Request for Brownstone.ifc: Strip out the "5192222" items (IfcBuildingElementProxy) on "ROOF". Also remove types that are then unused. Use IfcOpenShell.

First a look at what the model holds.

```python
import ifcopenshell
import ifcopenshell.util.element

model = ifcopenshell.open("Brownstone.ifc")
print(model.schema)
storey = next(s for s in model.by_type("IfcBuildingStorey") if s.Name == "ROOF")
proxies = [e for e in ifcopenshell.util.element.get_decomposition(storey) if e.is_a("IfcBuildingElementProxy")]
seen = {}
for e in proxies:
    element_type = ifcopenshell.util.element.get_type(e)
    name = element_type.Name if element_type not in (None, e) else None
    seen[name] = seen.get(name, 0) + 1
for name, count in sorted(seen.items(), key=str):
    print(count, "x", name)
```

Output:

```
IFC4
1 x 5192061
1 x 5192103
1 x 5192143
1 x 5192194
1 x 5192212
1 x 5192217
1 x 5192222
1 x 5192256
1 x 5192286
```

```python
import ifcopenshell
import ifcopenshell.api.root
import ifcopenshell.util.element

model = ifcopenshell.open("Brownstone.ifc")

storey = next(s for s in model.by_type("IfcBuildingStorey") if s.Name == "ROOF")
proxies = [e for e in ifcopenshell.util.element.get_decomposition(storey) if e.is_a("IfcBuildingElementProxy")]
targets = [e for e in proxies if (t := ifcopenshell.util.element.get_type(e)) not in (None, e) and t.Name == "5192222"]
types = {ifcopenshell.util.element.get_type(e) for e in targets} - {None, *targets}

for e in targets:
    ifcopenshell.api.root.remove_product(model, product=e)
print(len(targets), "removed")

unused = [t for t in types if not ifcopenshell.util.element.get_types(t)]
for t in unused:
    ifcopenshell.api.root.remove_product(model, product=t)
print(len(unused), "unused types removed")

model.write("Brownstone_v2.ifc")
```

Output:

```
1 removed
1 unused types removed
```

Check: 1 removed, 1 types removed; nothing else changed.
